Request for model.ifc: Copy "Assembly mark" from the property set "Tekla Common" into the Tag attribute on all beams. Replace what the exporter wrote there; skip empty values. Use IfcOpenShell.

First a look at what the model holds.

```python
import ifcopenshell
import ifcopenshell.util.element

model = ifcopenshell.open("model.ifc")
print(model.schema)
beams = model.by_type("IfcBeam")
print(len(beams), "beams")
for e in beams[:8]:
    source = ifcopenshell.util.element.get_pset(e, "Tekla Common", "Assembly mark")
    target = e.Tag
    print(e.id(), repr(source), repr(target), sep=" | ")
```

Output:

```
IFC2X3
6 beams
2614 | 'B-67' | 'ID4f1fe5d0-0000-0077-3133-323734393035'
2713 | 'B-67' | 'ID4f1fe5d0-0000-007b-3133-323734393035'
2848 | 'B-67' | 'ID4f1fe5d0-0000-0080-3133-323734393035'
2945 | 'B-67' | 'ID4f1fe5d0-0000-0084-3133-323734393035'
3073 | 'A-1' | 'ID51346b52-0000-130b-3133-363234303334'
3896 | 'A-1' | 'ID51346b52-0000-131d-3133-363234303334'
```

```python
import ifcopenshell
import ifcopenshell.util.element

model = ifcopenshell.open("model.ifc")

count = 0
for e in model.by_type("IfcBeam"):
    value = ifcopenshell.util.element.get_pset(e, "Tekla Common", "Assembly mark")
    current = e.Tag
    if not value or not value.strip() or current == value:
        continue
    e.Tag = value
    count += 1

print(count, "beams updated")

model.write("model-out.ifc")
```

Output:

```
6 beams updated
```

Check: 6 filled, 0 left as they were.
